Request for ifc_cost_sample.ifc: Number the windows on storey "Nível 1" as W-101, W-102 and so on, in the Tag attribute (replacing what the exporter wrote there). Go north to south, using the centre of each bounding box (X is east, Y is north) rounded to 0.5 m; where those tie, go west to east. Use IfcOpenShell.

First a look at what the model holds.

```python
import ifcopenshell
import ifcopenshell.util.element
import ifcopenshell.util.placement

model = ifcopenshell.open("ifc_cost_sample.ifc")
print(model.schema)
storey = next(s for s in model.by_type("IfcBuildingStorey") if s.Name == "Nível 1")
windows = [e for e in ifcopenshell.util.element.get_decomposition(storey) if e.is_a("IfcWindow")]
for e in sorted(windows, key=lambda e: e.id()):
    origin = ifcopenshell.util.placement.get_local_placement(e.ObjectPlacement)[:3, 3]
    print(e.id(), e.Tag, e.Name, origin.round(2) + 0.0, sep=" | ")
```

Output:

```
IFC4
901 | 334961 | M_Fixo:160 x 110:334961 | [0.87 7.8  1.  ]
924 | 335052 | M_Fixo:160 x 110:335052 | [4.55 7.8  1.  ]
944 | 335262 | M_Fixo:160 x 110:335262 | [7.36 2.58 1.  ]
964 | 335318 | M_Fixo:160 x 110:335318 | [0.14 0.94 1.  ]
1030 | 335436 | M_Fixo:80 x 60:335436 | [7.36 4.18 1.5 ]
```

```python
import ifcopenshell
import ifcopenshell.geom
import ifcopenshell.util.element
import ifcopenshell.util.shape

model = ifcopenshell.open("ifc_cost_sample.ifc")
settings = ifcopenshell.geom.settings()
settings.set("use-world-coords", True)


def centre(element):
    shape = ifcopenshell.geom.create_shape(settings, element)
    return ifcopenshell.util.shape.get_bbox_centroid(shape.geometry)


storey = next(s for s in model.by_type("IfcBuildingStorey") if s.Name == "Nível 1")
windows = [e for e in ifcopenshell.util.element.get_decomposition(storey) if e.is_a("IfcWindow")]

# Insertion points can sit at a corner or the storey origin, so sort by the geometry (in metres).
centres = {e: centre(e) for e in windows}
windows.sort(key=lambda e: (-round(centres[e][1] / 0.5), centres[e][0]))

for i, e in enumerate(windows, start=1):
    number = f"W-1{i:02d}"
    e.Tag = number
    print(e.id(), number)

model.write("ifc_cost_sample_updated.ifc")
```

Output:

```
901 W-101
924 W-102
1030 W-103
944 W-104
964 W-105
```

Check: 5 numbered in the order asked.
